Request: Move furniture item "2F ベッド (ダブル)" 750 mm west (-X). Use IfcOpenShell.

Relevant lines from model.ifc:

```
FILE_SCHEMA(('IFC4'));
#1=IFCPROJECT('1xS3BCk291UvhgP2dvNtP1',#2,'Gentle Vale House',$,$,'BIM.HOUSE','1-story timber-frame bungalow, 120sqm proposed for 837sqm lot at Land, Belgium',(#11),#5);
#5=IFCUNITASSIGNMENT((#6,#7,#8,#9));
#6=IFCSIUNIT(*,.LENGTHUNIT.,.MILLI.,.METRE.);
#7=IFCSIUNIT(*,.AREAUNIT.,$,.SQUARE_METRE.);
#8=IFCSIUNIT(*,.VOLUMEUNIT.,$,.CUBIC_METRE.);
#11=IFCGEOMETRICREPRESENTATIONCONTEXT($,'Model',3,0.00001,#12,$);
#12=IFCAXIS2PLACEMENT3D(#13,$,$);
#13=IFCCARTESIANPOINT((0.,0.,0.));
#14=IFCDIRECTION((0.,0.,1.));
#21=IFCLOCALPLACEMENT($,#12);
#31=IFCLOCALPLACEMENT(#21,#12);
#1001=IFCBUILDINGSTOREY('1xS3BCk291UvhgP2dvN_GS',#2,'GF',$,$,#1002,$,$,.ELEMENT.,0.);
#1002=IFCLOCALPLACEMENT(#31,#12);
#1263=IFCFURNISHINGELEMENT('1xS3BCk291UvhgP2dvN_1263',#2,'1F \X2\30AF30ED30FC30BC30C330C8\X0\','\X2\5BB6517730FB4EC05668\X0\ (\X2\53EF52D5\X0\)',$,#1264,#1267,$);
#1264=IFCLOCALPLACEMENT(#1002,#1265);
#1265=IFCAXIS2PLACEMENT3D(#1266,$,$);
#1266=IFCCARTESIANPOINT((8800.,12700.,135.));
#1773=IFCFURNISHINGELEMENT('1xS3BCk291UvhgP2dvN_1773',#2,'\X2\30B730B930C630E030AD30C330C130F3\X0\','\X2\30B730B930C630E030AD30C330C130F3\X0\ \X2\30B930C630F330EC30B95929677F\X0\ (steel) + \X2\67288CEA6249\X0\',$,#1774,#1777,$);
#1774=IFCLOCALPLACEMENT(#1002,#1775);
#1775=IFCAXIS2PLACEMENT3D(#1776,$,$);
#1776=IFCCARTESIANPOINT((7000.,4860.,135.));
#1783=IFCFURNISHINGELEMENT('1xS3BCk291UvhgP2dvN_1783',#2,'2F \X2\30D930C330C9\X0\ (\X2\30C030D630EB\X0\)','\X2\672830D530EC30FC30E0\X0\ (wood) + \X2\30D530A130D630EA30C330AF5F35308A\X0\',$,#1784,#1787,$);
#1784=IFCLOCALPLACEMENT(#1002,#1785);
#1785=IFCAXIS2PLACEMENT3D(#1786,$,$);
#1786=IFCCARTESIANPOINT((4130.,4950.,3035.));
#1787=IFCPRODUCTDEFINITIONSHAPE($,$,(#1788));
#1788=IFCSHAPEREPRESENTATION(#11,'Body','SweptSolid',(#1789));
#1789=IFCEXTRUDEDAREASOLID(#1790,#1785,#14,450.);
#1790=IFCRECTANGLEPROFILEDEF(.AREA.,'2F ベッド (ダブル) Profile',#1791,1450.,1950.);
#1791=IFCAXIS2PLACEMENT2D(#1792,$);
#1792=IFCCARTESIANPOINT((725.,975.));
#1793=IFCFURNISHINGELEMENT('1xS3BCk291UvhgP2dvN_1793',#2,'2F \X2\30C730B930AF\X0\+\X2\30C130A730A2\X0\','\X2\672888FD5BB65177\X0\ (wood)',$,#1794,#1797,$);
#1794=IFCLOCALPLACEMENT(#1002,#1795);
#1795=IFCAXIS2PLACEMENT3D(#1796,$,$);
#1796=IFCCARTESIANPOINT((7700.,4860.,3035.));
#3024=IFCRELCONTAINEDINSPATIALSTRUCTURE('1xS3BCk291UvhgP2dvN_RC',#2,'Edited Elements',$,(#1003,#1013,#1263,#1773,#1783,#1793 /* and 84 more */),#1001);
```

```python
import ifcopenshell
import ifcopenshell.api.geometry
import ifcopenshell.util.placement
import ifcopenshell.util.unit

model = ifcopenshell.open("model.ifc")
unit_scale = ifcopenshell.util.unit.calculate_unit_scale(model)

item = model.by_guid("1xS3BCk291UvhgP2dvN_1783")
matrix = ifcopenshell.util.placement.get_local_placement(item.ObjectPlacement)
matrix[0, 3] -= 0.75 / unit_scale
ifcopenshell.api.geometry.edit_object_placement(model, product=item, matrix=matrix, is_si=False)

print(ifcopenshell.util.placement.get_local_placement(item.ObjectPlacement).round(3) + 0.0)

model.write("model_v2.ifc")
```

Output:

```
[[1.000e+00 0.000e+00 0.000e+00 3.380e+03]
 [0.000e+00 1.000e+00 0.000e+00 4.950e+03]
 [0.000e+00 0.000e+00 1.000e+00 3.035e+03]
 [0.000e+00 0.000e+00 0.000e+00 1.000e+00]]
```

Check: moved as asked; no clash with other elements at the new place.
